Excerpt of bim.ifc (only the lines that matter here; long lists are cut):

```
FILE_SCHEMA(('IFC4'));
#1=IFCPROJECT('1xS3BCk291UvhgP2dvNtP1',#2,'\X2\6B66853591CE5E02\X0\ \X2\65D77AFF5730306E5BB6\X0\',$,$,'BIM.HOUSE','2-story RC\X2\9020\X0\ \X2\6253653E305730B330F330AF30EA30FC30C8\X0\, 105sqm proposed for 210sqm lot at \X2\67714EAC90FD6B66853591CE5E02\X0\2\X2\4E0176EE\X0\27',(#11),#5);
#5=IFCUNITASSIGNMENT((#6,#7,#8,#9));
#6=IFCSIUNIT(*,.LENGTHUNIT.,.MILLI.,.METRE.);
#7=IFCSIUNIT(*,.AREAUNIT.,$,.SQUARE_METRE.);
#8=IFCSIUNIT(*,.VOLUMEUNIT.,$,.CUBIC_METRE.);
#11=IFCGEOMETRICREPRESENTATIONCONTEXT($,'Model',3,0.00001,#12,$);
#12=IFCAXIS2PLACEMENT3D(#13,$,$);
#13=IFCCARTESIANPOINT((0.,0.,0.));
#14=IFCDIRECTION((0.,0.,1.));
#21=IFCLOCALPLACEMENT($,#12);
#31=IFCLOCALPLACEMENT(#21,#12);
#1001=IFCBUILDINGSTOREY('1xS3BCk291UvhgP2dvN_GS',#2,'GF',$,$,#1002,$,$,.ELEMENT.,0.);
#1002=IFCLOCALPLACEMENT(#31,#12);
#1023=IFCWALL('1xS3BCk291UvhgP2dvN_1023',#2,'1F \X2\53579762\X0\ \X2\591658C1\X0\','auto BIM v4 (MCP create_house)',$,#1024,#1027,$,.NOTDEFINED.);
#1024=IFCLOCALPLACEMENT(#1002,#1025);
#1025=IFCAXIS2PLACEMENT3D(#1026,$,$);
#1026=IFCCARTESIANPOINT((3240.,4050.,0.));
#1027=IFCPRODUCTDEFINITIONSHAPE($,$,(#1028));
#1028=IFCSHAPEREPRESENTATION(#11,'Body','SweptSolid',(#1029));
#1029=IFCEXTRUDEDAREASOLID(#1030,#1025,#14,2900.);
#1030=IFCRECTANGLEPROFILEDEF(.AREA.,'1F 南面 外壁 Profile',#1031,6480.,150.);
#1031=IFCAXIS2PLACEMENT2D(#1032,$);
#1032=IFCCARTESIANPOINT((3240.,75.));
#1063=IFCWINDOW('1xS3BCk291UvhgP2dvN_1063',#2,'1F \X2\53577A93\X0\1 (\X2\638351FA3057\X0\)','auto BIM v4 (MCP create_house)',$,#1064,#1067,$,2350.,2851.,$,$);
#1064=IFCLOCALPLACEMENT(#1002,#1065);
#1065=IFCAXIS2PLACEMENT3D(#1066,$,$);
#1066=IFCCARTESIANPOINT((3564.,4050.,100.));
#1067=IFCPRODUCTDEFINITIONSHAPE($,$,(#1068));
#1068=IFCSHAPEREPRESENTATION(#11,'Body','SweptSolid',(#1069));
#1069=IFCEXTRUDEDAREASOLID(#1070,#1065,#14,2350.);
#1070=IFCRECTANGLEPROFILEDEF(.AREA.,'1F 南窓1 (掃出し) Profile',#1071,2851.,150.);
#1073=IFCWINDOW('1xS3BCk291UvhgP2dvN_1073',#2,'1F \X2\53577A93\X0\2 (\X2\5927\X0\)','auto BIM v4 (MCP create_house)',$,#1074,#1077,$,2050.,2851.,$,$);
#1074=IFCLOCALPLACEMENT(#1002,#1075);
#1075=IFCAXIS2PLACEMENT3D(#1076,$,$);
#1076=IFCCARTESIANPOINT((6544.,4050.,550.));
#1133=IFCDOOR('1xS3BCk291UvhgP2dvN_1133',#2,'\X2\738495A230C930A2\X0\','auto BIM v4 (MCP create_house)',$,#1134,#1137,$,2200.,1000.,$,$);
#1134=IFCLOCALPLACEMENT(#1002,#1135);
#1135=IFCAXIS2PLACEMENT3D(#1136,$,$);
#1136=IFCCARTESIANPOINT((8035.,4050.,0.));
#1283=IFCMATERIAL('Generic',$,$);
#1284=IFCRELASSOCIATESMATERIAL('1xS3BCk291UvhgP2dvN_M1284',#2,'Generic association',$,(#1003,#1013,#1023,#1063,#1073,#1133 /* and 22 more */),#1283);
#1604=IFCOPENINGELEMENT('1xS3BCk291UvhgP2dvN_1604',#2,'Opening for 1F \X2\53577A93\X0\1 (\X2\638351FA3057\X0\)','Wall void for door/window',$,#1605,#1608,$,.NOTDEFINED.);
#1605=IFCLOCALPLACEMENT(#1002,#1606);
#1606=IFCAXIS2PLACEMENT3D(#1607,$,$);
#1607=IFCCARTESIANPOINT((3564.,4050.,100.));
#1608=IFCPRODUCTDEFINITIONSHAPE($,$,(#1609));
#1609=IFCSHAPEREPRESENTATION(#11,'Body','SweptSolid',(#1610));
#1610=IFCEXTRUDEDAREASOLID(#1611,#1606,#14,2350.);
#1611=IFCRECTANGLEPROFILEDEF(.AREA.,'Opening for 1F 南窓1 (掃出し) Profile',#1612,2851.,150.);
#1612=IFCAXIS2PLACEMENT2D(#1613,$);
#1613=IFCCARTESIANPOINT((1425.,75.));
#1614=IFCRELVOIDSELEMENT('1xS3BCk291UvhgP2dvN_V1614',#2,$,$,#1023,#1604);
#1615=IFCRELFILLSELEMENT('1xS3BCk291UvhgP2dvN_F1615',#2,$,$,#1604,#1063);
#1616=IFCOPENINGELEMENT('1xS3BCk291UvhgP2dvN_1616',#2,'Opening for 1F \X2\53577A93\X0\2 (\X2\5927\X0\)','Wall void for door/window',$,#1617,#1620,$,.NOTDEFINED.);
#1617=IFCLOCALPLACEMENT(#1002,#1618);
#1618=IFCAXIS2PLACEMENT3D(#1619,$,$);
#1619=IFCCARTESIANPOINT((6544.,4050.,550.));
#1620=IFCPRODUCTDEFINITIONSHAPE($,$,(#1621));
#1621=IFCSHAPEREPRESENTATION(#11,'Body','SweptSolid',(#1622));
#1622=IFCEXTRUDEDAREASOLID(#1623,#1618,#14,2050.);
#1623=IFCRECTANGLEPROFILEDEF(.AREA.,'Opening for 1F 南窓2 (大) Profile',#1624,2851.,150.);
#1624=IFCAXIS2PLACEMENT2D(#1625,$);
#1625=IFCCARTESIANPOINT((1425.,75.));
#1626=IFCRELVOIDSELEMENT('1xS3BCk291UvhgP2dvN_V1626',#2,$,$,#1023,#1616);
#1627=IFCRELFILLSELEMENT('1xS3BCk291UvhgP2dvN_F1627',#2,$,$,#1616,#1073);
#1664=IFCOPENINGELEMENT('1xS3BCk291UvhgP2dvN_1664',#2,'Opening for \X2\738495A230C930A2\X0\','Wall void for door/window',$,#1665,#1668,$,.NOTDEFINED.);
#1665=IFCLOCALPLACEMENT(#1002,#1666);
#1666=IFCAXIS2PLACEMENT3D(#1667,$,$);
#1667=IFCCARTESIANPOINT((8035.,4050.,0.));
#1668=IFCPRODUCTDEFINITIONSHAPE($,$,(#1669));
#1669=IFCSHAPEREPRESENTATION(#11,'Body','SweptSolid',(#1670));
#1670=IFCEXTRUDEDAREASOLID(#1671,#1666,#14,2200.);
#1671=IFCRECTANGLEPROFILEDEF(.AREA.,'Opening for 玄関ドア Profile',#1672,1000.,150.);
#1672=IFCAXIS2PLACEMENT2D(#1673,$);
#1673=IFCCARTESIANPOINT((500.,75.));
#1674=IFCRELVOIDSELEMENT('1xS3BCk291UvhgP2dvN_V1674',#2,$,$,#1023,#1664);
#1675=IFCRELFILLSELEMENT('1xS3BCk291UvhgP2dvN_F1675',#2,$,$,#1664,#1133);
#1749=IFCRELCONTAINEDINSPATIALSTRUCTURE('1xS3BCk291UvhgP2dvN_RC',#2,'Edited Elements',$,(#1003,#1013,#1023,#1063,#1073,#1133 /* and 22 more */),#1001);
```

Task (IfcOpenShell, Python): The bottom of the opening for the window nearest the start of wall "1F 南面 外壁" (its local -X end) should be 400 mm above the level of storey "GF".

```python
import numpy as np
import ifcopenshell
import ifcopenshell.api.geometry
import ifcopenshell.geom
import ifcopenshell.util.element
import ifcopenshell.util.placement
import ifcopenshell.util.shape
import ifcopenshell.util.unit

model = ifcopenshell.open("bim.ifc")
unit_scale = ifcopenshell.util.unit.calculate_unit_scale(model)

window = model.by_guid("1xS3BCk291UvhgP2dvN_1063")
opening = window.FillsVoids[0].RelatingOpeningElement
storey = ifcopenshell.util.element.get_container(window, ifc_class="IfcBuildingStorey")
level = ifcopenshell.util.placement.get_local_placement(storey.ObjectPlacement)[2, 3]

# The opening's origin need not be at the sill, so measure its lowest point.
shape = ifcopenshell.geom.create_shape(ifcopenshell.geom.settings(), opening)
bottom = ifcopenshell.util.shape.get_shape_bottom_elevation(shape, shape.geometry) / unit_scale
dz = level + 0.4 / unit_scale - bottom

shift = np.array([0.0, 0.0, dz])
# The window is not placed relative to its opening, so move both.
for product in (opening, window):
    matrix = ifcopenshell.util.placement.get_local_placement(product.ObjectPlacement)
    matrix[:3, 3] += shift
    ifcopenshell.api.geometry.edit_object_placement(model, product=product, matrix=matrix, is_si=False)

print(f"moved by {dz * unit_scale:+.3f} m")

model.write("bim_rev.ifc")
```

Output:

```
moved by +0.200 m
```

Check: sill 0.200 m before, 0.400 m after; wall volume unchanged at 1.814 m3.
